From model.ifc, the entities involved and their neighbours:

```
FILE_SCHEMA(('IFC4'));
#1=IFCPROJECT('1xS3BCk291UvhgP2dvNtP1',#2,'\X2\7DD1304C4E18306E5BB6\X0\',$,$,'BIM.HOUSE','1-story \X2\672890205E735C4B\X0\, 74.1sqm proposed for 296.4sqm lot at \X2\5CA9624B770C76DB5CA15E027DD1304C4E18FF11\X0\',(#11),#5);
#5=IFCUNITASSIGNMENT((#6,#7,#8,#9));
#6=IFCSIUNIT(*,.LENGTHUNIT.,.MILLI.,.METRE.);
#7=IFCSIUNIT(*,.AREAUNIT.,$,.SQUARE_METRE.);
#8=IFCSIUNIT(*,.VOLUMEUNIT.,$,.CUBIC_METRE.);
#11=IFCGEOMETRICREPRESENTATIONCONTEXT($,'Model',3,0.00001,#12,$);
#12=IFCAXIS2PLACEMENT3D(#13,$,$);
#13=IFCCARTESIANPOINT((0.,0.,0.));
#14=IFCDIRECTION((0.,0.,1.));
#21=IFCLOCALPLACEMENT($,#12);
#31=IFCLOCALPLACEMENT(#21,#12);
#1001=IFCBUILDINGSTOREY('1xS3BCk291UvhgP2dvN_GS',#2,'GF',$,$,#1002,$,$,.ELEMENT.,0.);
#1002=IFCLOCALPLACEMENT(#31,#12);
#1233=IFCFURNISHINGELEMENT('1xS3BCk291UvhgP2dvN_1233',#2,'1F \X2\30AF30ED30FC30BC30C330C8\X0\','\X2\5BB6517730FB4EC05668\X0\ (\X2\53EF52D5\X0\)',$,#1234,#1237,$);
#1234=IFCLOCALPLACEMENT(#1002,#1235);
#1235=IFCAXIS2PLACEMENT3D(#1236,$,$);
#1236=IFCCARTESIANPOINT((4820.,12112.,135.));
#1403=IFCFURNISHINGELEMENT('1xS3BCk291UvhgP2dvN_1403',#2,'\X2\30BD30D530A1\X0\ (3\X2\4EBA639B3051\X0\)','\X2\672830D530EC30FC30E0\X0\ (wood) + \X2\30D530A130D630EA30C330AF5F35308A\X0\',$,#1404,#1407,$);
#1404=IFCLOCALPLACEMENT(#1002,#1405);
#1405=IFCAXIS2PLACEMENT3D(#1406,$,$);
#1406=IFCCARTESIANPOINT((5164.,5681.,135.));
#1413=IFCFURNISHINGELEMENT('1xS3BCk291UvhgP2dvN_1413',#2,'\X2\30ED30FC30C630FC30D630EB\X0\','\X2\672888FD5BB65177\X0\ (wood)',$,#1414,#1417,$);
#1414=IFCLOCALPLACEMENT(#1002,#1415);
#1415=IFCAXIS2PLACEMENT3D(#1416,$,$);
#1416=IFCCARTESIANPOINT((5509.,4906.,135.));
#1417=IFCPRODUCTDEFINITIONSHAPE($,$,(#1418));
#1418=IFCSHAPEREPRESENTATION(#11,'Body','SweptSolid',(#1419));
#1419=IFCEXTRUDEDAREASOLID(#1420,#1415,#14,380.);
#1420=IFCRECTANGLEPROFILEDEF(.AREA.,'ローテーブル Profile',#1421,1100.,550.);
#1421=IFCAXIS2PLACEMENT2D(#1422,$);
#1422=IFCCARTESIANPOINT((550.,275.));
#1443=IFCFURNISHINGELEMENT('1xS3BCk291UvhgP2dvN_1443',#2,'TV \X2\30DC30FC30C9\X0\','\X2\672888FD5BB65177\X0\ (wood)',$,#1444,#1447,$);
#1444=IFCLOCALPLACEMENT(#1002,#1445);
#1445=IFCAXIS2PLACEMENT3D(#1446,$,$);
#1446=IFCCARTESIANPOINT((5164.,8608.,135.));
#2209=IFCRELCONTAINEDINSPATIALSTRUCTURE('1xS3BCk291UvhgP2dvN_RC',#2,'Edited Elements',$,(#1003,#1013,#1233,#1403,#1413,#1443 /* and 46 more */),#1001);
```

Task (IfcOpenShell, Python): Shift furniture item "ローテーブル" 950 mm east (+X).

```python
import ifcopenshell
import ifcopenshell.api.geometry
import ifcopenshell.util.placement

model = ifcopenshell.open("model.ifc")

item = model.by_guid("1xS3BCk291UvhgP2dvN_1413")
matrix = ifcopenshell.util.placement.get_local_placement(item.ObjectPlacement)
matrix[0, 3] += 950.0
ifcopenshell.api.geometry.edit_object_placement(model, product=item, matrix=matrix, is_si=False)

print(ifcopenshell.util.placement.get_local_placement(item.ObjectPlacement).round(3) + 0.0)

model.write("model-out.ifc")
```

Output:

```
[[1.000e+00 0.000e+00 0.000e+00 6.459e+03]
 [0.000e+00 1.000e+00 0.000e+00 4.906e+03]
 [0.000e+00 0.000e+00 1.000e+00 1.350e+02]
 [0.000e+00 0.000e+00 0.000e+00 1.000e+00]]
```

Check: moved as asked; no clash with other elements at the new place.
